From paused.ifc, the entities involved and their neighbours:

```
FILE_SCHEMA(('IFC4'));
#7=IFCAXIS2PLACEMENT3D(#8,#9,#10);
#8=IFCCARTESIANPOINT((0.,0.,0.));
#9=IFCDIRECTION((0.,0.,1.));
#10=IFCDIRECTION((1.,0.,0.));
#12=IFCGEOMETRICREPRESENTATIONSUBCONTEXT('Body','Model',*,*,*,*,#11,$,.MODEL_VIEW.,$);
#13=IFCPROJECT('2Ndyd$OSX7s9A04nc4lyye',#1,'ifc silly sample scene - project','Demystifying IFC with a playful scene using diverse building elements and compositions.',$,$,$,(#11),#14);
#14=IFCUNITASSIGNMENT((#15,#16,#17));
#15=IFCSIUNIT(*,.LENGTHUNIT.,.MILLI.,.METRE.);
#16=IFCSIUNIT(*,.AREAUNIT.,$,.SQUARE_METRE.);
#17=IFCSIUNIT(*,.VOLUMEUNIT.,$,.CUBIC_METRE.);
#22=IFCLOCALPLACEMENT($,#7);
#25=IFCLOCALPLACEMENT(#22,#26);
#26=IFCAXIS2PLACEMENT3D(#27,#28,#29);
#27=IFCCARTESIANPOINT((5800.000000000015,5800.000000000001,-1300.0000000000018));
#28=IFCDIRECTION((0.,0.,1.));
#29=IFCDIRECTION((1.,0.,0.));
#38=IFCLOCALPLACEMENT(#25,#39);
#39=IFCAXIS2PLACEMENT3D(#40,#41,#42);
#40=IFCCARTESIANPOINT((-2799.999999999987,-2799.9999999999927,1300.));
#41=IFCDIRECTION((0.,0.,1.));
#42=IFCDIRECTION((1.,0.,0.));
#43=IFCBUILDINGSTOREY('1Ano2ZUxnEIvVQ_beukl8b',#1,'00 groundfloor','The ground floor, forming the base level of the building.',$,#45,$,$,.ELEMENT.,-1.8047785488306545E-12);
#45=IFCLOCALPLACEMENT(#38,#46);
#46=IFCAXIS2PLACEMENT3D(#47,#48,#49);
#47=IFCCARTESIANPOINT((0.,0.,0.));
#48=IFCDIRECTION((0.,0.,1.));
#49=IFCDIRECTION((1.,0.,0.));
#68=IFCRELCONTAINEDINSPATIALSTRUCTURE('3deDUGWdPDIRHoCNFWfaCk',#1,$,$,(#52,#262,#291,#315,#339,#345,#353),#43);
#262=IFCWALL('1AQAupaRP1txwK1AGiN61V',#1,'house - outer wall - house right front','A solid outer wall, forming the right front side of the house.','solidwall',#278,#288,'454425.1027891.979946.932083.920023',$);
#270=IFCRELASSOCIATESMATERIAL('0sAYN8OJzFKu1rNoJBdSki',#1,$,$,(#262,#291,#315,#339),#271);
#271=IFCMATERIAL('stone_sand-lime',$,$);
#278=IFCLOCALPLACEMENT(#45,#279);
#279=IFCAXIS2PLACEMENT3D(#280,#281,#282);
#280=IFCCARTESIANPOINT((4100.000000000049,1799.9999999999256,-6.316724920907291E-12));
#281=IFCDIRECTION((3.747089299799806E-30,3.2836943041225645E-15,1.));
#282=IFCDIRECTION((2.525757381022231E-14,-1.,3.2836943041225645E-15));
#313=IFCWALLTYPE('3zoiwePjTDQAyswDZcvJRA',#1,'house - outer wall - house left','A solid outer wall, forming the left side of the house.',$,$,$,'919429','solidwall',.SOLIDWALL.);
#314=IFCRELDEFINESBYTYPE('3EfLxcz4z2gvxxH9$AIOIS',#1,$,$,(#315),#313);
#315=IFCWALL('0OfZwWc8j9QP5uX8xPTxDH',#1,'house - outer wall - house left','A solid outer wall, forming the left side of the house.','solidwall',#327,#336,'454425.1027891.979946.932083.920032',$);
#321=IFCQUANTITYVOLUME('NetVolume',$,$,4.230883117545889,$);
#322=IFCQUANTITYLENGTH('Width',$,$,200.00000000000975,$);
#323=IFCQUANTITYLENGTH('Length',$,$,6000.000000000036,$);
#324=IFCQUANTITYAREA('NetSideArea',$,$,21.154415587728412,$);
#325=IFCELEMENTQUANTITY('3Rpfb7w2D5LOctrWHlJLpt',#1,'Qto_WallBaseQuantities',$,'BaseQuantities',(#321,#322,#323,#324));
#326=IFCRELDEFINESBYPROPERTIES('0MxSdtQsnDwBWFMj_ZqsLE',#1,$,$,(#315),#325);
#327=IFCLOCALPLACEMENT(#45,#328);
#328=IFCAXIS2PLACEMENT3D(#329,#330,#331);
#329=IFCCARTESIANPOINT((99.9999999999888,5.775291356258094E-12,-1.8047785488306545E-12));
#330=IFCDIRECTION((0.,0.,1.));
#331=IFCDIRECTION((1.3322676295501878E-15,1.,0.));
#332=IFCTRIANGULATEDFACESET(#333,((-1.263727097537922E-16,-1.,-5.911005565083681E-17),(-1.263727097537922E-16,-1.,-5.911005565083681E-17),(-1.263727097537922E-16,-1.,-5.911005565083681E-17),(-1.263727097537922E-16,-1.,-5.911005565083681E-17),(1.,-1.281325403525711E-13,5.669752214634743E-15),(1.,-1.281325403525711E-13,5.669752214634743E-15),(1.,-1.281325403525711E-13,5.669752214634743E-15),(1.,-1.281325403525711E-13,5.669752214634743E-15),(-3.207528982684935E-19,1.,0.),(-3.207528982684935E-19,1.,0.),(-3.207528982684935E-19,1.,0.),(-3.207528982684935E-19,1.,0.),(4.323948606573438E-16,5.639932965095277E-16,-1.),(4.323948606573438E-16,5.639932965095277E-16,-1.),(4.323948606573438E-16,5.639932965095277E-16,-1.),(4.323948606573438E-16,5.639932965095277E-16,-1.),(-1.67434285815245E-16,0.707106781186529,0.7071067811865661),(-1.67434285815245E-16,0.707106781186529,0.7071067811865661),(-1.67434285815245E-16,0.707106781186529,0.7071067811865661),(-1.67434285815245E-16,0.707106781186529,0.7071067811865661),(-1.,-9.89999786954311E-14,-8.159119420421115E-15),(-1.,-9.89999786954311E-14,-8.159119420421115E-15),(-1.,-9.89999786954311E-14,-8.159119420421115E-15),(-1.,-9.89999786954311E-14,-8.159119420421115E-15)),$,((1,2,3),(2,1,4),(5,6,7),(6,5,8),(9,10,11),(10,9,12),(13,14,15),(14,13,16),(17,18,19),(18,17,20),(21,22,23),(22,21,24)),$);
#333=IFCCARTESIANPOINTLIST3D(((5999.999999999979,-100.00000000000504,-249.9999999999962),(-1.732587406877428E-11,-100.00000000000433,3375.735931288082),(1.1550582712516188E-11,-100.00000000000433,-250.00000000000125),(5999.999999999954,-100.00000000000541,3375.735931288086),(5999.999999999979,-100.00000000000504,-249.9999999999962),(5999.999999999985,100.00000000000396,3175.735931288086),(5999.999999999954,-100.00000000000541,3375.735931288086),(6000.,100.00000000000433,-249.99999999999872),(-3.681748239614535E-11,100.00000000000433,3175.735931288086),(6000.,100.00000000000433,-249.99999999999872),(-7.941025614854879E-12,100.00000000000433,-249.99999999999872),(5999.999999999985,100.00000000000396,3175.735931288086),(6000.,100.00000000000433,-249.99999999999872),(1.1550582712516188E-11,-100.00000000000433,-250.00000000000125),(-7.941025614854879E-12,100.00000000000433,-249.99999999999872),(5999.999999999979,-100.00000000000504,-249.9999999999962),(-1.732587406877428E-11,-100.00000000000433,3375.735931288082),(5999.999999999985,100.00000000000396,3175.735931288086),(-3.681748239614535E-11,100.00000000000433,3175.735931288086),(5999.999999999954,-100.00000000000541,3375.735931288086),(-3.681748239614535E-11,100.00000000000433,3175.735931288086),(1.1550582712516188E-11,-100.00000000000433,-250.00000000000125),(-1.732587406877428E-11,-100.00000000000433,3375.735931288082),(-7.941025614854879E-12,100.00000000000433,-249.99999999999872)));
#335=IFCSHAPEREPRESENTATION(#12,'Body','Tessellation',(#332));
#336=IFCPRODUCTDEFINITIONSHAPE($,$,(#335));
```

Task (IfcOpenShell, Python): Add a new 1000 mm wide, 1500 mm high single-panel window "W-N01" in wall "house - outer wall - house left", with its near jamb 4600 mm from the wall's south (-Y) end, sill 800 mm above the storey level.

```python
import numpy as np
import ifcopenshell
import ifcopenshell.api.feature
import ifcopenshell.api.geometry
import ifcopenshell.api.pset
import ifcopenshell.api.root
import ifcopenshell.api.spatial
import ifcopenshell.geom
import ifcopenshell.util.element
import ifcopenshell.util.placement
import ifcopenshell.util.representation
import ifcopenshell.util.shape
import ifcopenshell.util.unit

model = ifcopenshell.open("paused.ifc")
unit_scale = ifcopenshell.util.unit.calculate_unit_scale(model)
area_scale = ifcopenshell.util.unit.calculate_unit_scale(model, "AREAUNIT")
volume_scale = ifcopenshell.util.unit.calculate_unit_scale(model, "VOLUMEUNIT")
settings = ifcopenshell.geom.settings()


def volume(element):
    """Net volume in cubic metres, openings subtracted."""
    shape = ifcopenshell.geom.create_shape(settings, element)
    return ifcopenshell.util.shape.get_volume(shape.geometry)


wall = model.by_guid("0OfZwWc8j9QP5uX8xPTxDH")
storey = ifcopenshell.util.element.get_container(wall, ifc_class="IfcBuildingStorey")
context = ifcopenshell.util.representation.get_context(model, "Model", "Body", "MODEL_VIEW")
before = volume(wall)

width, height, from_end, sill = 1, 1.5, 4.6, 0.8  # metres

# The wall runs along its own X axis, and the end named is its -X end.
wall_shape = ifcopenshell.geom.create_shape(settings, wall)
x, y, z = ifcopenshell.util.shape.get_vertices(wall_shape.geometry).T
start = x.min() + from_end
face, thickness = float(y.min()), float(y.max() - y.min())
wall_matrix = ifcopenshell.util.placement.get_local_placement(wall.ObjectPlacement)
level = ifcopenshell.util.placement.get_local_placement(storey.ObjectPlacement)[2, 3]


def in_wall(x, y):
    """Placement at x, y metres in the wall's axes, at sill height."""
    matrix = wall_matrix.copy()
    matrix[:, 3] = wall_matrix @ np.array([x / unit_scale, y / unit_scale, 0.0, 1.0])
    matrix[2, 3] = level + sill / unit_scale
    return matrix


# Opening: a box that overshoots both wall faces by 50 mm.
opening = ifcopenshell.api.root.create_entity(model, ifc_class="IfcOpeningElement", predefined_type="OPENING")
box = ifcopenshell.api.geometry.add_wall_representation(
    model, context=context, length=width, height=height, thickness=thickness + 0.1
)
ifcopenshell.api.geometry.assign_representation(model, product=opening, representation=box)
ifcopenshell.api.geometry.edit_object_placement(model, product=opening, matrix=in_wall(start, face - 0.05), is_si=False)
ifcopenshell.api.feature.add_feature(model, feature=opening, element=wall)

window = ifcopenshell.api.root.create_entity(model, ifc_class="IfcWindow", name="W-N01", predefined_type="WINDOW")
window.OverallWidth, window.OverallHeight = width / unit_scale, height / unit_scale
window.PartitioningType = "SINGLE_PANEL"
body = ifcopenshell.api.geometry.add_window_representation(
    model,
    context=context,
    overall_width=window.OverallWidth,
    overall_height=window.OverallHeight,
    partition_type="SINGLE_PANEL",
)
ifcopenshell.api.geometry.assign_representation(model, product=window, representation=body)
ifcopenshell.api.spatial.assign_container(model, products=[window], relating_structure=storey)
ifcopenshell.api.feature.add_filling(model, opening=opening, element=window)

# Centre the window in the wall's thickness.
ifcopenshell.api.geometry.edit_object_placement(model, product=window, matrix=in_wall(start, face), is_si=False)
window_shape = ifcopenshell.geom.create_shape(settings, window)
depth = ifcopenshell.util.shape.get_vertices(window_shape.geometry)[:, 1]
offset = face + thickness / 2 - (depth.min() + depth.max()) / 2
ifcopenshell.api.geometry.edit_object_placement(model, product=window, matrix=in_wall(start, offset), is_si=False)

after = volume(wall)

# Update the wall's stored quantities.
qto = model.by_id(ifcopenshell.util.element.get_pset(wall, "Qto_WallBaseQuantities", should_inherit=False)["id"])
ifcopenshell.api.pset.edit_qto(model, qto=qto, properties={
    "NetVolume": after / volume_scale,
    "NetSideArea": after / thickness / area_scale,
})

print(f"wall volume {before:.3f} -> {after:.3f} m3")

model.write("paused_edited.ifc")
```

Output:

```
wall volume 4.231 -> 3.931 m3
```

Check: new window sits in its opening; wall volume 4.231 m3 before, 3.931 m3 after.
